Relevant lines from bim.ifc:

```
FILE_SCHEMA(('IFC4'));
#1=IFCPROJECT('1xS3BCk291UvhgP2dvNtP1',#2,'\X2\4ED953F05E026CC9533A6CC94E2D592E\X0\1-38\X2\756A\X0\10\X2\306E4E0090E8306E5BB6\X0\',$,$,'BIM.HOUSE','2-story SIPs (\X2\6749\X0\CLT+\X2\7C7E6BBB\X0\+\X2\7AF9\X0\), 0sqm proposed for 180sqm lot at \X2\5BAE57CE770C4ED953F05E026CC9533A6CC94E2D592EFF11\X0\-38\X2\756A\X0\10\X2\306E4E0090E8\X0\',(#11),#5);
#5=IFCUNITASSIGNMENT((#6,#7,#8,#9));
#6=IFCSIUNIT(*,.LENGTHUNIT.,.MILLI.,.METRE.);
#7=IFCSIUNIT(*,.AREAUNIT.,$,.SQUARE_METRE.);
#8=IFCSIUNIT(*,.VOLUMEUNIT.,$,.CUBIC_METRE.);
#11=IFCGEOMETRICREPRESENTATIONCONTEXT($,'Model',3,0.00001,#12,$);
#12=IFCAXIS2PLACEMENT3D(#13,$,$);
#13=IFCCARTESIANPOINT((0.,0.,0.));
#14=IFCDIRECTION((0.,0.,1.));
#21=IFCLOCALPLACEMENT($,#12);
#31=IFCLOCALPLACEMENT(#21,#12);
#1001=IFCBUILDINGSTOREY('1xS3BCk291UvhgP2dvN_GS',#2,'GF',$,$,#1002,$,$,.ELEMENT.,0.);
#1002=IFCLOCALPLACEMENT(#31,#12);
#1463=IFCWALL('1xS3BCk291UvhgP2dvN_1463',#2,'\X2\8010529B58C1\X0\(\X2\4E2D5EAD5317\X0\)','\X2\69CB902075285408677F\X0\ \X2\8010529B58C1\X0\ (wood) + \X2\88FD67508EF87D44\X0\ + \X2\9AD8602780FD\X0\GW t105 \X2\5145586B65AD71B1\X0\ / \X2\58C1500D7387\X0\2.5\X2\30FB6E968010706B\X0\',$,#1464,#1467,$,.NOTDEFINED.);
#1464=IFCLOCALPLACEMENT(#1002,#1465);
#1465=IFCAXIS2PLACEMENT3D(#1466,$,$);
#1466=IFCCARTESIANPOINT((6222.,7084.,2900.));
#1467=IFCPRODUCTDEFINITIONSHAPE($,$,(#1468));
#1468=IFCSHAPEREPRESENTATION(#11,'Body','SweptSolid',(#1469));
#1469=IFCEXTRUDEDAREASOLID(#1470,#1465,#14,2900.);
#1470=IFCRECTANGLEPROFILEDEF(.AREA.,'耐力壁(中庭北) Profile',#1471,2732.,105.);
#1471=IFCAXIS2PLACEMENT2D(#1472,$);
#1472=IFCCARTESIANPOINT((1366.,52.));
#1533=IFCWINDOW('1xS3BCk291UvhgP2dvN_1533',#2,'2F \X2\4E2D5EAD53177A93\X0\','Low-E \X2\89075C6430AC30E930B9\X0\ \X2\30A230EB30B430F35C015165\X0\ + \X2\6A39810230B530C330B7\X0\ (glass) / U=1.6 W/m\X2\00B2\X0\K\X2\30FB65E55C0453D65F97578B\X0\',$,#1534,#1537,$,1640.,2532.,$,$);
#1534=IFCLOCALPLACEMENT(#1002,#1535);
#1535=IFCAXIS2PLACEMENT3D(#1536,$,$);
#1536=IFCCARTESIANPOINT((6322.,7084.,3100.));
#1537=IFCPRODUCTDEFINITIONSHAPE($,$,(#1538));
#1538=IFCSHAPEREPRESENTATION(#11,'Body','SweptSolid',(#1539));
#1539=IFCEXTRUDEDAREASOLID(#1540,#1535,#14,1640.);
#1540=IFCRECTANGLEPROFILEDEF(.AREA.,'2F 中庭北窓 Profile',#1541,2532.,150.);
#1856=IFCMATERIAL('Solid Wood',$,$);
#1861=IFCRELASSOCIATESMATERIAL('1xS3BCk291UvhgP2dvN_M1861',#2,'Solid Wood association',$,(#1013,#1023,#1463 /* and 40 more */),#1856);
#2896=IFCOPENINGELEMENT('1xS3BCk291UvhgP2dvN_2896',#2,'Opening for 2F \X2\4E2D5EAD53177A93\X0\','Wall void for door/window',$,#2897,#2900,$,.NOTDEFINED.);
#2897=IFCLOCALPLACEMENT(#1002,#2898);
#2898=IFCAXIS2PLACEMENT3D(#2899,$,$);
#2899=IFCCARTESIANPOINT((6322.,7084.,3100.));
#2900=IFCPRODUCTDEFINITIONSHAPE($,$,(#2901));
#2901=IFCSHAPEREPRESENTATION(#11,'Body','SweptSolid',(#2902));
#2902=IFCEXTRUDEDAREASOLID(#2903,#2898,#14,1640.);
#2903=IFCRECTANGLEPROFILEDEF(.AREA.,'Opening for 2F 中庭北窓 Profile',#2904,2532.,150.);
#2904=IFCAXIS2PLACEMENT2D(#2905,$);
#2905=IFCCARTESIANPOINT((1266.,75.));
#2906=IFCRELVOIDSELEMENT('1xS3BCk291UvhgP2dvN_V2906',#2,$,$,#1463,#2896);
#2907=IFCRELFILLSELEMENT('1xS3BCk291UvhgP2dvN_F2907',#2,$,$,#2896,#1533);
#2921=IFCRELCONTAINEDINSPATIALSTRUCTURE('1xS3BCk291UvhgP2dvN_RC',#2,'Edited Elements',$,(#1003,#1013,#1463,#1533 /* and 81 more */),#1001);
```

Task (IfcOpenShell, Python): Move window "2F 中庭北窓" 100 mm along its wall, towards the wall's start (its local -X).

```python
import ifcopenshell
import ifcopenshell.api.geometry
import ifcopenshell.util.placement

model = ifcopenshell.open("bim.ifc")

window = model.by_guid("1xS3BCk291UvhgP2dvN_1533")
opening = window.FillsVoids[0].RelatingOpeningElement
wall = opening.VoidsElements[0].RelatingBuildingElement

wall_matrix = ifcopenshell.util.placement.get_local_placement(wall.ObjectPlacement)
shift = wall_matrix[:3, 0] * -100.0
before = ifcopenshell.util.placement.get_local_placement(window.ObjectPlacement)[:3, 3].copy()

# The window is not placed relative to its opening, so move both.
for product in (opening, window):
    matrix = ifcopenshell.util.placement.get_local_placement(product.ObjectPlacement)
    matrix[:3, 3] += shift
    ifcopenshell.api.geometry.edit_object_placement(model, product=product, matrix=matrix, is_si=False)

after = ifcopenshell.util.placement.get_local_placement(window.ObjectPlacement)[:3, 3]
print("window moved by", (after - before).round(3) + 0.0)

model.write("bim_edited.ifc")
```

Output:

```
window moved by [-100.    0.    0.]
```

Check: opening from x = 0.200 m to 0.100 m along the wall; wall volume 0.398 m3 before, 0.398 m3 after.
